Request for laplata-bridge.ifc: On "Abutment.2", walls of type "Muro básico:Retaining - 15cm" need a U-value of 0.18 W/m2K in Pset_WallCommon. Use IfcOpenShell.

First a look at what the model holds.

```python
import ifcopenshell
import ifcopenshell.util.element

model = ifcopenshell.open("laplata-bridge.ifc")
print(model.schema)
storey = next(s for s in model.by_type("IfcBuildingStorey") if s.Name == "Abutment.2")
walls = [e for e in ifcopenshell.util.element.get_decomposition(storey) if e.is_a("IfcWall")]
seen = {}
for e in walls:
    element_type = ifcopenshell.util.element.get_type(e)
    key = (element_type.Name if element_type != e and element_type else None, ifcopenshell.util.element.get_pset(e, "Pset_WallCommon", "ThermalTransmittance"))
    seen[key] = seen.get(key, 0) + 1
for (name, value), count in sorted(seen.items(), key=str):
    print(count, "x", name, "|", value)
```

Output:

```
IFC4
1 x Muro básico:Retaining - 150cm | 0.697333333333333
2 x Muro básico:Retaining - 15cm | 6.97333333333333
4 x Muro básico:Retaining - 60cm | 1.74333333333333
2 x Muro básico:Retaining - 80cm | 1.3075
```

```python
import ifcopenshell
import ifcopenshell.api.pset
import ifcopenshell.util.element

model = ifcopenshell.open("laplata-bridge.ifc")

storey = next(s for s in model.by_type("IfcBuildingStorey") if s.Name == "Abutment.2")
walls = [e for e in ifcopenshell.util.element.get_decomposition(storey) if e.is_a("IfcWall")]

count = 0
for e in walls:
    element_type = ifcopenshell.util.element.get_type(e)
    if element_type in (None, e) or element_type.Name != "Muro básico:Retaining - 15cm":
        continue
    # add_pset returns the element's existing set when there is one.
    pset = ifcopenshell.api.pset.add_pset(model, product=e, name="Pset_WallCommon")
    ifcopenshell.api.pset.edit_pset(model, pset=pset, properties={"ThermalTransmittance": 0.18})
    count += 1

print(count, "walls updated")

model.write("laplata-bridge-out.ifc")
```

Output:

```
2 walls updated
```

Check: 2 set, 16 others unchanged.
